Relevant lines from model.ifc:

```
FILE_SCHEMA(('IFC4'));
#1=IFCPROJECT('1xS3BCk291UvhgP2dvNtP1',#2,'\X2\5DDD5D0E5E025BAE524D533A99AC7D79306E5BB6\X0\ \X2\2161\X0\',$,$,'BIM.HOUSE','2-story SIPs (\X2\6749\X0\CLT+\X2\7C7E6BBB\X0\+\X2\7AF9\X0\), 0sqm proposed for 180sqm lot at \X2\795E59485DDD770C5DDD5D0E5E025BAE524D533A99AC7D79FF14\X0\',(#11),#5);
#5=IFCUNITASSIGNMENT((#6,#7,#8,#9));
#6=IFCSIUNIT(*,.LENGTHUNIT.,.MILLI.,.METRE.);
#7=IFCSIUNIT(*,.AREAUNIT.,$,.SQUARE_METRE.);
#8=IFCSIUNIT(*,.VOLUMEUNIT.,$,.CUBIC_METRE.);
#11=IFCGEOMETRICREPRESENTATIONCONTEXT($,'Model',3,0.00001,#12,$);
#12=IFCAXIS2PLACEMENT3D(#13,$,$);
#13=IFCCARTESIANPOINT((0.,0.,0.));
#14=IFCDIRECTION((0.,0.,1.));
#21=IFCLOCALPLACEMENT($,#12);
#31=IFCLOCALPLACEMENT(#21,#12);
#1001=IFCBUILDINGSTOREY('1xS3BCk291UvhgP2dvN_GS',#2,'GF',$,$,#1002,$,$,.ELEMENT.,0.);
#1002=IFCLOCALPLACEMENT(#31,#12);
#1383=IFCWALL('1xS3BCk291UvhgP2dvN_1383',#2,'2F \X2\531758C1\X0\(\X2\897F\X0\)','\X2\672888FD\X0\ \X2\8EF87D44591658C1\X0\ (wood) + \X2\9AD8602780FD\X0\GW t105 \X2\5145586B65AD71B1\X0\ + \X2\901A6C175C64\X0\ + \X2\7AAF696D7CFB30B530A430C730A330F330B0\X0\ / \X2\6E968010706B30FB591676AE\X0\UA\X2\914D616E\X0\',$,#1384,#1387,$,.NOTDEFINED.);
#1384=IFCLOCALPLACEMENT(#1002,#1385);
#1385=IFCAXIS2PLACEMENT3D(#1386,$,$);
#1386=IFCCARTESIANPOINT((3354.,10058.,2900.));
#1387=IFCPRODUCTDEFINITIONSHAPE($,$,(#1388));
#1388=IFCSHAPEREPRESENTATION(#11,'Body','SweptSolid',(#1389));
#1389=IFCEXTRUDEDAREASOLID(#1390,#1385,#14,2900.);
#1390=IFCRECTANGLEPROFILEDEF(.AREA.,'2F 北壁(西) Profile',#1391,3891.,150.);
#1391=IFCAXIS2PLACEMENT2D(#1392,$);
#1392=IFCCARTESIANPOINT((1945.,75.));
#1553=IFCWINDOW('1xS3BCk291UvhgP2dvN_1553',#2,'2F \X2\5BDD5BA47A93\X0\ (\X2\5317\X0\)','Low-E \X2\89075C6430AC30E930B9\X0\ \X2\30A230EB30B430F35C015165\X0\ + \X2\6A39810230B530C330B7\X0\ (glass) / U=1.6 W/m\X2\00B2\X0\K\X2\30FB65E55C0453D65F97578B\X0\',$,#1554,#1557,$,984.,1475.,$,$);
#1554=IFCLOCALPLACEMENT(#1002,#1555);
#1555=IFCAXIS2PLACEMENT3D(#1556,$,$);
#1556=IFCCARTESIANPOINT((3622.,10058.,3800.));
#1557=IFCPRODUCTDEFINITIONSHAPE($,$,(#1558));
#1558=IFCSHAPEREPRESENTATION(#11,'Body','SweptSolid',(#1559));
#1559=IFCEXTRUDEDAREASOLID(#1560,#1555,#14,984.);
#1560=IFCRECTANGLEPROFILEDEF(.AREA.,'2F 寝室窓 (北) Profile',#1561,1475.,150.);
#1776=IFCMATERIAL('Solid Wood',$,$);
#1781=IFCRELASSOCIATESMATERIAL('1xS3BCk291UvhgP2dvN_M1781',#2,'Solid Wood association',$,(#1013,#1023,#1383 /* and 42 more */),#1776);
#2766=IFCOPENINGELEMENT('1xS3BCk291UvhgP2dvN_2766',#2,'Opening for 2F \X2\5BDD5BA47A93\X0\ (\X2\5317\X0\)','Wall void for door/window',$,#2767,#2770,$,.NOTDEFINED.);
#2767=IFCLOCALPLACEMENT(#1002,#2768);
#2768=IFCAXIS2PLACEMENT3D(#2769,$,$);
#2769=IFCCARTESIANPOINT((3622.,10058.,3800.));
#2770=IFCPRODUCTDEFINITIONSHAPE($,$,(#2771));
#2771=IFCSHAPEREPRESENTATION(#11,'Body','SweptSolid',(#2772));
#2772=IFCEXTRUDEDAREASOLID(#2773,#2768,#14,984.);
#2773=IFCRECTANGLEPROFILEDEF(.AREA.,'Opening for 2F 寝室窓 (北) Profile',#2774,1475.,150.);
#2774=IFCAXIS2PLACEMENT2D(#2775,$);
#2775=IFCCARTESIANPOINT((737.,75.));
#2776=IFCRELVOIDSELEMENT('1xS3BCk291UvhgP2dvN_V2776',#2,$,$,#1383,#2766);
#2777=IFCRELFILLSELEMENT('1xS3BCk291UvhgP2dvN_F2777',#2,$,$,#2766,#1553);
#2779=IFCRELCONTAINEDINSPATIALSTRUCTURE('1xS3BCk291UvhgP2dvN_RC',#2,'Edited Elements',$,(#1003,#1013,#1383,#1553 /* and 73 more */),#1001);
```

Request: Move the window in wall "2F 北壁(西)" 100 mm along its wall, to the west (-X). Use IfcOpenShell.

```python
import ifcopenshell
import ifcopenshell.api.geometry
import ifcopenshell.util.placement
import ifcopenshell.util.unit

model = ifcopenshell.open("model.ifc")
unit_scale = ifcopenshell.util.unit.calculate_unit_scale(model)

window = model.by_guid("1xS3BCk291UvhgP2dvN_1553")
opening = window.FillsVoids[0].RelatingOpeningElement
wall = opening.VoidsElements[0].RelatingBuildingElement

wall_matrix = ifcopenshell.util.placement.get_local_placement(wall.ObjectPlacement)
shift = wall_matrix[:3, 0] * -0.1 / unit_scale
before = ifcopenshell.util.placement.get_local_placement(window.ObjectPlacement)[:3, 3].copy()

# The window is not placed relative to its opening, so move both.
for product in (opening, window):
    matrix = ifcopenshell.util.placement.get_local_placement(product.ObjectPlacement)
    matrix[:3, 3] += shift
    ifcopenshell.api.geometry.edit_object_placement(model, product=product, matrix=matrix, is_si=False)

after = ifcopenshell.util.placement.get_local_placement(window.ObjectPlacement)[:3, 3]
print("window moved by", (after - before).round(3) + 0.0)

model.write("model_rev.ifc")
```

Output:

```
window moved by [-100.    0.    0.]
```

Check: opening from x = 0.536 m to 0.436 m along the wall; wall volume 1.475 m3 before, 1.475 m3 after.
